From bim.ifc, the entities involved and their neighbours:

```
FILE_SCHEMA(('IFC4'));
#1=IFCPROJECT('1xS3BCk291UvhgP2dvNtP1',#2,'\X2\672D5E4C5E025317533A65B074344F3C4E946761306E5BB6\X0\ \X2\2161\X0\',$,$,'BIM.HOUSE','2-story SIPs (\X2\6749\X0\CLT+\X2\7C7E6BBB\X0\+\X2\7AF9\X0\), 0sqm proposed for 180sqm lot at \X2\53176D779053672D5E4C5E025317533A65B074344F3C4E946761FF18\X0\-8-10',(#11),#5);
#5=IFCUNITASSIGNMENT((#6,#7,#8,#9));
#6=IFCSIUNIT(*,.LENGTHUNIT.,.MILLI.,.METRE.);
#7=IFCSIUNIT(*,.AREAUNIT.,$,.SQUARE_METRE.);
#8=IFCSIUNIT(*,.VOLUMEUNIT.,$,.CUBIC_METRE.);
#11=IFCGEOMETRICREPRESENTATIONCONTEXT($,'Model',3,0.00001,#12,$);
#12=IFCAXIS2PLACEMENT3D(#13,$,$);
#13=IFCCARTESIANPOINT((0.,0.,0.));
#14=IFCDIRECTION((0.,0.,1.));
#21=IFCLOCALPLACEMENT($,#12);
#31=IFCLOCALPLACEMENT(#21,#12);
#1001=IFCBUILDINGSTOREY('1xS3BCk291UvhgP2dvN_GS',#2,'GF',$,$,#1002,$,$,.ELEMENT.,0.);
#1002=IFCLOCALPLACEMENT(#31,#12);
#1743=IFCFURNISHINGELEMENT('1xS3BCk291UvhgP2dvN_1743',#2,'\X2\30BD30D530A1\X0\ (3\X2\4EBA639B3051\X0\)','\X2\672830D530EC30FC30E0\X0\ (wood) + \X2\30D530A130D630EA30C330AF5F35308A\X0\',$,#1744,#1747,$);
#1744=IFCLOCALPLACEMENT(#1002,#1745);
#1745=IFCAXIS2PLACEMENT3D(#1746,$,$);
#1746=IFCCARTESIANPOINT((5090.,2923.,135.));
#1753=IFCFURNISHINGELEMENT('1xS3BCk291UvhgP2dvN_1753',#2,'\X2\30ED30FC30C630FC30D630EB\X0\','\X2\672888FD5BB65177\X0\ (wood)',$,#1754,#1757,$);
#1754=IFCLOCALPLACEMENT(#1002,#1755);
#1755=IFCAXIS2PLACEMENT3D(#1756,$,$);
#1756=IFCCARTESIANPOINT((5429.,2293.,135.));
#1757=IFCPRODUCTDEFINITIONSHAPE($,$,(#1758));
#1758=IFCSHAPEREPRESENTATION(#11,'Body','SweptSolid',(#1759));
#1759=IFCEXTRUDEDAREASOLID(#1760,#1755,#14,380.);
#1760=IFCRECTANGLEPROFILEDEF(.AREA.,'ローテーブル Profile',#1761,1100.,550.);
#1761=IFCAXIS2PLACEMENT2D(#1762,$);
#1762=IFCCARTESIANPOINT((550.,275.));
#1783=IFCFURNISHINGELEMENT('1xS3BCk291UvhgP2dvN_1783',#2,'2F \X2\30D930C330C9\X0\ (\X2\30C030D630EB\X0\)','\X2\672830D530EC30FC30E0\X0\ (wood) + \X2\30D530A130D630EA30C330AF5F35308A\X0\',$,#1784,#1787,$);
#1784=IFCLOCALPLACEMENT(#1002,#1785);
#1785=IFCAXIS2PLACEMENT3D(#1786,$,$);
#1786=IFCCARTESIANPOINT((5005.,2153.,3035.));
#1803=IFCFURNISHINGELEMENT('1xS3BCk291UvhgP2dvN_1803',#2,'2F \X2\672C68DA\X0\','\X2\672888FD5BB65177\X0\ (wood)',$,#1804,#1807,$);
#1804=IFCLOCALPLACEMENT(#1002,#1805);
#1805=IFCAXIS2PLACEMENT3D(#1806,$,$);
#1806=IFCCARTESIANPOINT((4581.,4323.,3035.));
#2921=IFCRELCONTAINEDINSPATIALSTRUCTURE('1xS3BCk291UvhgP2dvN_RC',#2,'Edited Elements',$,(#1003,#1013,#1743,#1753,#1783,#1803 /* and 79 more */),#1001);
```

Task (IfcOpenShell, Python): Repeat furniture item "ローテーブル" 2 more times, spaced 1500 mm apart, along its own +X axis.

```python
import ifcopenshell
import ifcopenshell.api.geometry
import ifcopenshell.api.root
import ifcopenshell.util.element
import ifcopenshell.util.placement
import ifcopenshell.util.unit

model = ifcopenshell.open("bim.ifc")
unit_scale = ifcopenshell.util.unit.calculate_unit_scale(model)


def reuse_history(source, copy):
    """copy_class also copies each property set's owner history, people and application; keep the originals."""
    for rel in copy.IsDefinedBy:
        if rel.is_a("IfcRelDefinesByProperties") and (history := rel.RelatingPropertyDefinition.OwnerHistory):
            rel.RelatingPropertyDefinition.OwnerHistory = source.OwnerHistory
            ifcopenshell.util.element.remove_deep2(model, history)


source = model.by_guid("1xS3BCk291UvhgP2dvN_1753")
base = ifcopenshell.util.placement.get_local_placement(source.ObjectPlacement)
step = base[:3, 0] * 1.5 / unit_scale

for i in range(1, 3):
    copy = ifcopenshell.api.root.copy_class(model, product=source)
    copy.Representation = ifcopenshell.util.element.copy_deep(
        model, source.Representation, exclude=["IfcGeometricRepresentationContext", "IfcRepresentationMap"]
    )
    reuse_history(source, copy)
    matrix = base.copy()
    matrix[:3, 3] += i * step
    print("added at", matrix[:3, 3].round(3) + 0.0)
    ifcopenshell.api.geometry.edit_object_placement(model, product=copy, matrix=matrix, is_si=False)

model.write("bim_updated.ifc")
```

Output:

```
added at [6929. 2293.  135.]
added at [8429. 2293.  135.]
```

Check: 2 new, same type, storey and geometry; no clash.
